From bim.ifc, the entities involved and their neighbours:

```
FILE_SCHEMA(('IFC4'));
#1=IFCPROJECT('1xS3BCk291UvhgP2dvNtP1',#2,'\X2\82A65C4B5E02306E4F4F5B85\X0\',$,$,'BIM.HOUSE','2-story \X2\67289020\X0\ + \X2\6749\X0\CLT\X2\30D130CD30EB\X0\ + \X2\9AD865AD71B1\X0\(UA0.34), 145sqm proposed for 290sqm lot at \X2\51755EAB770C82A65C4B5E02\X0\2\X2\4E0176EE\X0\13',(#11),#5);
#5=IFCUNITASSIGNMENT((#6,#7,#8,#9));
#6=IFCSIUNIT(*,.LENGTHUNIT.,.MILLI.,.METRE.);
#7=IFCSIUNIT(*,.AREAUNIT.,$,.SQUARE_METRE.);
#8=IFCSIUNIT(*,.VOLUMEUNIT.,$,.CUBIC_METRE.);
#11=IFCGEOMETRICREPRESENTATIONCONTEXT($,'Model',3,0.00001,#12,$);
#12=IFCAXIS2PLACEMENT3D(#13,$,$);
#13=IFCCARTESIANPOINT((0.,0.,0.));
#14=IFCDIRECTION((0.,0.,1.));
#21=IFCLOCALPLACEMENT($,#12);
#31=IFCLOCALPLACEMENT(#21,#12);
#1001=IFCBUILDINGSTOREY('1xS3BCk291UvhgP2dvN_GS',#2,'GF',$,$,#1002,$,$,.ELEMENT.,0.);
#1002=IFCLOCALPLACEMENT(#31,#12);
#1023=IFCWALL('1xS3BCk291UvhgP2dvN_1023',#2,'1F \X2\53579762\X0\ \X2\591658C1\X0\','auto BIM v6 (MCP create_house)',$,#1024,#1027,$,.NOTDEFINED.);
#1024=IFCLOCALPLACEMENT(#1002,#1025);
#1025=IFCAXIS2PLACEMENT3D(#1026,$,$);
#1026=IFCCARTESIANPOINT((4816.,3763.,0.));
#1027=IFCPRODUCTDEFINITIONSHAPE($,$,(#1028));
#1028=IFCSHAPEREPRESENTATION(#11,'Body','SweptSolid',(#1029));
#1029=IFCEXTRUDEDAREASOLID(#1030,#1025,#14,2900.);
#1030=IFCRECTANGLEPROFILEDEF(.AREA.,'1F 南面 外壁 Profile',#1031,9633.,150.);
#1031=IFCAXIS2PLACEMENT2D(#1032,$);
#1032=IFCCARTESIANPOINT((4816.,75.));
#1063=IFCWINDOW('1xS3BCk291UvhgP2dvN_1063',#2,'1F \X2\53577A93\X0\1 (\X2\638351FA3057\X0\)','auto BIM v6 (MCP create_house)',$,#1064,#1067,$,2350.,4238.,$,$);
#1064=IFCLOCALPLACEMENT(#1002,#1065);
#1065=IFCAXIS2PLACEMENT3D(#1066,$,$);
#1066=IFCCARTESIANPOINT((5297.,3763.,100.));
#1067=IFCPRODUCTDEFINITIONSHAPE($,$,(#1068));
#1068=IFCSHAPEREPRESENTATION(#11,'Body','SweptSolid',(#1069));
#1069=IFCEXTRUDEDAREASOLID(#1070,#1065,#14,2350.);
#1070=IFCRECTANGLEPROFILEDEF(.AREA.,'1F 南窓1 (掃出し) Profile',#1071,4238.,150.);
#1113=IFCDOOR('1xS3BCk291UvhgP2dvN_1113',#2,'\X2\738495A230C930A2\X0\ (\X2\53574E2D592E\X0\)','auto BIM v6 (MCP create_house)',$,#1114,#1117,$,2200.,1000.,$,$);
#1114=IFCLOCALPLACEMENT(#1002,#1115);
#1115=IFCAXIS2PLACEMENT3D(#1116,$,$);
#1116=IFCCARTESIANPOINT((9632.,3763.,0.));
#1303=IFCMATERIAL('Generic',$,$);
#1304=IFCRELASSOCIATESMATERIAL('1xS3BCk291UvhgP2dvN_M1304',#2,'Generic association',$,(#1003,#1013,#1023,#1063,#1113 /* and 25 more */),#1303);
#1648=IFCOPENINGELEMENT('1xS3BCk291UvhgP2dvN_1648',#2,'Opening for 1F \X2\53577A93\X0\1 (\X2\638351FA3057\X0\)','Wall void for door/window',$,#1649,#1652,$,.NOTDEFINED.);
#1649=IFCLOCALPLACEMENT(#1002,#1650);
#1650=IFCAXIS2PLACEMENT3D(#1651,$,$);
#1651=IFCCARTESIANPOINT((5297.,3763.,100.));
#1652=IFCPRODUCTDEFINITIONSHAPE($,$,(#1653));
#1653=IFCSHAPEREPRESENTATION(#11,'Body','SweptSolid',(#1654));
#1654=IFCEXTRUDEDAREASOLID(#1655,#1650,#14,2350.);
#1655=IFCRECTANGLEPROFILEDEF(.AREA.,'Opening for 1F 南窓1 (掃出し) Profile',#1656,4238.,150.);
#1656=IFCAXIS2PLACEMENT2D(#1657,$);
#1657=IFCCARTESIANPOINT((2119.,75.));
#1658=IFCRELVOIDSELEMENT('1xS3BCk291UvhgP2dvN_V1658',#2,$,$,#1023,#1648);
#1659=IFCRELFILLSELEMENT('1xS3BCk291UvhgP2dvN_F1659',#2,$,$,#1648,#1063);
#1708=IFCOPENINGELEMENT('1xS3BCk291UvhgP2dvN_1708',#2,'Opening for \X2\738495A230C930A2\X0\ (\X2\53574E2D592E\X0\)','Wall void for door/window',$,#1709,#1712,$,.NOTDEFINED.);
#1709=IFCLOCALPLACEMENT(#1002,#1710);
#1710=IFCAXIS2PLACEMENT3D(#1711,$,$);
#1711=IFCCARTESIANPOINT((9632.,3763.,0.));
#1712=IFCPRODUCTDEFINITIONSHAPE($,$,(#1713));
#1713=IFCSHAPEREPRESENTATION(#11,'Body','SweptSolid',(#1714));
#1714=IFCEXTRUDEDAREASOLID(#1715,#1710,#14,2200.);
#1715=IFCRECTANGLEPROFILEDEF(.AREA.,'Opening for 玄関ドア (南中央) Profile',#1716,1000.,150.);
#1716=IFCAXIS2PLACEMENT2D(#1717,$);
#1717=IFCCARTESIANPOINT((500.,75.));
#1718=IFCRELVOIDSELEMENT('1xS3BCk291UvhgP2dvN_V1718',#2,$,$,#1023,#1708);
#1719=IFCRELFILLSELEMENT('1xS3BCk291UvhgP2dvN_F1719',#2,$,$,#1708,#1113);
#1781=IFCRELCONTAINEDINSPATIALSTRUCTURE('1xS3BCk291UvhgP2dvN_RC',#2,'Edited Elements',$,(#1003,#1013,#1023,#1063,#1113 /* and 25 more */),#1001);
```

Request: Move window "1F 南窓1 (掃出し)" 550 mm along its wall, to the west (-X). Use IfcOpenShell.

```python
import ifcopenshell
import ifcopenshell.api.geometry
import ifcopenshell.util.placement

model = ifcopenshell.open("bim.ifc")

window = model.by_guid("1xS3BCk291UvhgP2dvN_1063")
opening = window.FillsVoids[0].RelatingOpeningElement
wall = opening.VoidsElements[0].RelatingBuildingElement

wall_matrix = ifcopenshell.util.placement.get_local_placement(wall.ObjectPlacement)
shift = wall_matrix[:3, 0] * -550.0
before = ifcopenshell.util.placement.get_local_placement(window.ObjectPlacement)[:3, 3].copy()

# The window is not placed relative to its opening, so move both.
for product in (opening, window):
    matrix = ifcopenshell.util.placement.get_local_placement(product.ObjectPlacement)
    matrix[:3, 3] += shift
    ifcopenshell.api.geometry.edit_object_placement(model, product=product, matrix=matrix, is_si=False)

after = ifcopenshell.util.placement.get_local_placement(window.ObjectPlacement)[:3, 3]
print("window moved by", (after - before).round(3) + 0.0)

model.write("bim_v2.ifc")
```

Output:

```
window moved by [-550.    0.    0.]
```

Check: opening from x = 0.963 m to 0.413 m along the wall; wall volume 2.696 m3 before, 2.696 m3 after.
